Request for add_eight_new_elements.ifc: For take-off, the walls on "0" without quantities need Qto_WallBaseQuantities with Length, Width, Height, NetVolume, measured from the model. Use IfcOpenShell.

First a look at what the model holds.

```python
import ifcopenshell
import ifcopenshell.util.element
import ifcopenshell.util.unit

model = ifcopenshell.open("add_eight_new_elements.ifc")
print(model.schema)
for unit_type in ("LENGTHUNIT", "AREAUNIT", "VOLUMEUNIT"):
    print(unit_type, ifcopenshell.util.unit.calculate_unit_scale(model, unit_type))
storey = next(s for s in model.by_type("IfcBuildingStorey") if s.Name == "0")
walls = [e for e in ifcopenshell.util.element.get_decomposition(storey) if e.is_a("IfcWall")]
for e in sorted(walls, key=lambda e: e.id()):
    print(e.id(), e.is_a(), e.Name, list(ifcopenshell.util.element.get_psets(e, qtos_only=True)), sep=" | ")
```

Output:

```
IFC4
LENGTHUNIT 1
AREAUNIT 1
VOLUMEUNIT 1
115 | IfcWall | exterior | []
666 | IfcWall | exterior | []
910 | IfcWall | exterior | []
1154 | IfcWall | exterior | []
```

```python
import ifcopenshell
import ifcopenshell.api.pset
import ifcopenshell.geom
import ifcopenshell.util.element
import ifcopenshell.util.shape
import ifcopenshell.util.unit

model = ifcopenshell.open("add_eight_new_elements.ifc")
unit_scale = ifcopenshell.util.unit.calculate_unit_scale(model)
volume_scale = ifcopenshell.util.unit.calculate_unit_scale(model, "VOLUMEUNIT")
settings = ifcopenshell.geom.settings()

storey = next(s for s in model.by_type("IfcBuildingStorey") if s.Name == "0")
walls = [e for e in ifcopenshell.util.element.get_decomposition(storey) if e.is_a("IfcWall")]

for e in sorted(walls, key=lambda e: e.id()):
    if ifcopenshell.util.element.get_psets(e, qtos_only=True, should_inherit=False):
        continue
    # Geometry comes back in metres, in the element's own axes.
    shape = ifcopenshell.geom.create_shape(settings, e)
    values = {
        "Length": ifcopenshell.util.shape.get_x(shape.geometry) / unit_scale,
        "Width": ifcopenshell.util.shape.get_y(shape.geometry) / unit_scale,
        "Height": ifcopenshell.util.shape.get_z(shape.geometry) / unit_scale,
        "NetVolume": ifcopenshell.util.shape.get_volume(shape.geometry) / volume_scale,
    }
    qto = ifcopenshell.api.pset.add_qto(model, product=e, name="Qto_WallBaseQuantities")
    ifcopenshell.api.pset.edit_qto(model, qto=qto, properties=values)
    print(e.id(), {k: round(v, 3) for k, v in values.items()})

model.write("add_eight_new_elements_v2.ifc")
```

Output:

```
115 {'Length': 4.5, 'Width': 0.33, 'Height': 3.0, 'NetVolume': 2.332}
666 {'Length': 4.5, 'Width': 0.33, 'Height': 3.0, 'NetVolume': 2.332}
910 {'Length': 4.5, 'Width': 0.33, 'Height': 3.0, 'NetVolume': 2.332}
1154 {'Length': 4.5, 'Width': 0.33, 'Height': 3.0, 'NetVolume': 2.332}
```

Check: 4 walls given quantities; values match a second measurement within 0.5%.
